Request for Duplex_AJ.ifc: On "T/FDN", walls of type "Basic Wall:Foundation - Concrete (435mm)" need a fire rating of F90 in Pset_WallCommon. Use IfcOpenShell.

First a look at what the model holds.

```python
import ifcopenshell
import ifcopenshell.util.element

model = ifcopenshell.open("Duplex_AJ.ifc")
print(model.schema)
storey = next(s for s in model.by_type("IfcBuildingStorey") if s.Name == "T/FDN")
walls = [e for e in ifcopenshell.util.element.get_decomposition(storey) if e.is_a("IfcWall")]
seen = {}
for e in walls:
    element_type = ifcopenshell.util.element.get_type(e)
    key = (element_type.Name if element_type != e and element_type else None, ifcopenshell.util.element.get_pset(e, "Pset_WallCommon", "FireRating"))
    seen[key] = seen.get(key, 0) + 1
for (name, value), count in sorted(seen.items(), key=str):
    print(count, "x", name, "|", value)
```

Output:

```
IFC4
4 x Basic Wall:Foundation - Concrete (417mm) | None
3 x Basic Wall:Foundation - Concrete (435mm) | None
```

```python
import ifcopenshell
import ifcopenshell.api.pset
import ifcopenshell.util.element

model = ifcopenshell.open("Duplex_AJ.ifc")

storey = next(s for s in model.by_type("IfcBuildingStorey") if s.Name == "T/FDN")
walls = [e for e in ifcopenshell.util.element.get_decomposition(storey) if e.is_a("IfcWall")]

count = 0
for e in walls:
    element_type = ifcopenshell.util.element.get_type(e)
    if element_type in (None, e) or element_type.Name != "Basic Wall:Foundation - Concrete (435mm)":
        continue
    # add_pset returns the element's existing set when there is one.
    pset = ifcopenshell.api.pset.add_pset(model, product=e, name="Pset_WallCommon")
    ifcopenshell.api.pset.edit_pset(model, pset=pset, properties={"FireRating": "F90"})
    count += 1

print(count, "walls updated")

model.write("Duplex_AJ_updated.ifc")
```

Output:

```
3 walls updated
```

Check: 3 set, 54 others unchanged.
